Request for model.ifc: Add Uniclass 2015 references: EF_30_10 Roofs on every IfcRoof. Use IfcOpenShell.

First a look at what the model holds.

```python
import ifcopenshell

model = ifcopenshell.open("model.ifc")
print(model.schema)
print("classifications:", [c.Name for c in model.by_type("IfcClassification")])
for ifc_class in ("IfcDoor", "IfcRoof", "IfcStair", "IfcWall", "IfcWindow"):
    print(ifc_class, len(model.by_type(ifc_class)))
```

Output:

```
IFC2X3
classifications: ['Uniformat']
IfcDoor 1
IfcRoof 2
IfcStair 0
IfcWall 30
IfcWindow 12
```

```python
import ifcopenshell
import ifcopenshell.api.classification

model = ifcopenshell.open("model.ifc")

# IFC2X3 requires Source and Edition and has no link from the project to the system.
system = model.create_entity("IfcClassification", Source="NBS", Edition="2015", Name="Uniclass 2015")

codes = {
    "IfcRoof": ("EF_30_10", "Roofs"),
}
for ifc_class, (code, name) in codes.items():
    products = model.by_type(ifc_class)
    ifcopenshell.api.classification.add_reference(
        model, products=products, classification=system, identification=code, name=name
    )
    print(code, len(products))

model.write("model_rev.ifc")
```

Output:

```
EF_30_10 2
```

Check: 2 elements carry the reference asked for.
